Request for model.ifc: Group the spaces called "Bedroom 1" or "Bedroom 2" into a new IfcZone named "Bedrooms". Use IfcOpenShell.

First a look at what the model holds.

```python
import ifcopenshell

model = ifcopenshell.open("model.ifc")
print(model.schema)
seen = {}
for space in model.by_type("IfcSpace"):
    seen[space.LongName] = seen.get(space.LongName, 0) + 1
for name, count in sorted(seen.items(), key=str):
    print(count, "x", name)
print("zones:", [z.Name for z in model.by_type("IfcZone")][:20])
```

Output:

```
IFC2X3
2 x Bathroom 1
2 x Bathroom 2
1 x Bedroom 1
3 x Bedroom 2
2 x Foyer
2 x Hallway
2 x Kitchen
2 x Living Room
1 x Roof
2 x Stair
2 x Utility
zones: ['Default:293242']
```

```python
import ifcopenshell
import ifcopenshell.api.group
import ifcopenshell.api.root

model = ifcopenshell.open("model.ifc")

names = {"Bedroom 1", "Bedroom 2"}
spaces = [s for s in model.by_type("IfcSpace") if s.LongName in names]

zone = ifcopenshell.api.root.create_entity(model, ifc_class="IfcZone", name="Bedrooms")
ifcopenshell.api.group.assign_group(model, products=spaces, group=zone)
print(len(spaces), "spaces in", zone.Name)

model.write("model_edited.ifc")
```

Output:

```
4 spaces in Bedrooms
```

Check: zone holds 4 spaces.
